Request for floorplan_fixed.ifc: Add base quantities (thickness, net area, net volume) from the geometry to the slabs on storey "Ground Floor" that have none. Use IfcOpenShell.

First a look at what the model holds.

```python
import ifcopenshell
import ifcopenshell.util.element
import ifcopenshell.util.unit

model = ifcopenshell.open("floorplan_fixed.ifc")
print(model.schema)
for unit_type in ("LENGTHUNIT", "AREAUNIT", "VOLUMEUNIT"):
    print(unit_type, ifcopenshell.util.unit.calculate_unit_scale(model, unit_type))
storey = next(s for s in model.by_type("IfcBuildingStorey") if s.Name == "Ground Floor")
slabs = [e for e in ifcopenshell.util.element.get_decomposition(storey) if e.is_a("IfcSlab")]
for e in sorted(slabs, key=lambda e: e.id()):
    print(e.id(), e.is_a(), e.Name, list(ifcopenshell.util.element.get_psets(e, qtos_only=True)), sep=" | ")
```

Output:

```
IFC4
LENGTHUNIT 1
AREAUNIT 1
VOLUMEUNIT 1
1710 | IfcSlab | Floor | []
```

```python
import ifcopenshell
import ifcopenshell.api.pset
import ifcopenshell.geom
import ifcopenshell.util.element
import ifcopenshell.util.shape
import ifcopenshell.util.unit

model = ifcopenshell.open("floorplan_fixed.ifc")
unit_scale = ifcopenshell.util.unit.calculate_unit_scale(model)
area_scale = ifcopenshell.util.unit.calculate_unit_scale(model, "AREAUNIT")
volume_scale = ifcopenshell.util.unit.calculate_unit_scale(model, "VOLUMEUNIT")
settings = ifcopenshell.geom.settings()

storey = next(s for s in model.by_type("IfcBuildingStorey") if s.Name == "Ground Floor")
slabs = [e for e in ifcopenshell.util.element.get_decomposition(storey) if e.is_a("IfcSlab")]

for e in sorted(slabs, key=lambda e: e.id()):
    if ifcopenshell.util.element.get_psets(e, qtos_only=True, should_inherit=False):
        continue
    # Geometry comes back in metres, in the element's own axes.
    shape = ifcopenshell.geom.create_shape(settings, e)
    values = {
        "Width": ifcopenshell.util.shape.get_z(shape.geometry) / unit_scale,
        "NetArea": ifcopenshell.util.shape.get_footprint_area(shape.geometry) / area_scale,
        "NetVolume": ifcopenshell.util.shape.get_volume(shape.geometry) / volume_scale,
    }
    qto = ifcopenshell.api.pset.add_qto(model, product=e, name="Qto_SlabBaseQuantities")
    ifcopenshell.api.pset.edit_qto(model, qto=qto, properties=values)
    print(e.id(), {k: round(v, 3) for k, v in values.items()})

model.write("floorplan_fixed_v2.ifc")
```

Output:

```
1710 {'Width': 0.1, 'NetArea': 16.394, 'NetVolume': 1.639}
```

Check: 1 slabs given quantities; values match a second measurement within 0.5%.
